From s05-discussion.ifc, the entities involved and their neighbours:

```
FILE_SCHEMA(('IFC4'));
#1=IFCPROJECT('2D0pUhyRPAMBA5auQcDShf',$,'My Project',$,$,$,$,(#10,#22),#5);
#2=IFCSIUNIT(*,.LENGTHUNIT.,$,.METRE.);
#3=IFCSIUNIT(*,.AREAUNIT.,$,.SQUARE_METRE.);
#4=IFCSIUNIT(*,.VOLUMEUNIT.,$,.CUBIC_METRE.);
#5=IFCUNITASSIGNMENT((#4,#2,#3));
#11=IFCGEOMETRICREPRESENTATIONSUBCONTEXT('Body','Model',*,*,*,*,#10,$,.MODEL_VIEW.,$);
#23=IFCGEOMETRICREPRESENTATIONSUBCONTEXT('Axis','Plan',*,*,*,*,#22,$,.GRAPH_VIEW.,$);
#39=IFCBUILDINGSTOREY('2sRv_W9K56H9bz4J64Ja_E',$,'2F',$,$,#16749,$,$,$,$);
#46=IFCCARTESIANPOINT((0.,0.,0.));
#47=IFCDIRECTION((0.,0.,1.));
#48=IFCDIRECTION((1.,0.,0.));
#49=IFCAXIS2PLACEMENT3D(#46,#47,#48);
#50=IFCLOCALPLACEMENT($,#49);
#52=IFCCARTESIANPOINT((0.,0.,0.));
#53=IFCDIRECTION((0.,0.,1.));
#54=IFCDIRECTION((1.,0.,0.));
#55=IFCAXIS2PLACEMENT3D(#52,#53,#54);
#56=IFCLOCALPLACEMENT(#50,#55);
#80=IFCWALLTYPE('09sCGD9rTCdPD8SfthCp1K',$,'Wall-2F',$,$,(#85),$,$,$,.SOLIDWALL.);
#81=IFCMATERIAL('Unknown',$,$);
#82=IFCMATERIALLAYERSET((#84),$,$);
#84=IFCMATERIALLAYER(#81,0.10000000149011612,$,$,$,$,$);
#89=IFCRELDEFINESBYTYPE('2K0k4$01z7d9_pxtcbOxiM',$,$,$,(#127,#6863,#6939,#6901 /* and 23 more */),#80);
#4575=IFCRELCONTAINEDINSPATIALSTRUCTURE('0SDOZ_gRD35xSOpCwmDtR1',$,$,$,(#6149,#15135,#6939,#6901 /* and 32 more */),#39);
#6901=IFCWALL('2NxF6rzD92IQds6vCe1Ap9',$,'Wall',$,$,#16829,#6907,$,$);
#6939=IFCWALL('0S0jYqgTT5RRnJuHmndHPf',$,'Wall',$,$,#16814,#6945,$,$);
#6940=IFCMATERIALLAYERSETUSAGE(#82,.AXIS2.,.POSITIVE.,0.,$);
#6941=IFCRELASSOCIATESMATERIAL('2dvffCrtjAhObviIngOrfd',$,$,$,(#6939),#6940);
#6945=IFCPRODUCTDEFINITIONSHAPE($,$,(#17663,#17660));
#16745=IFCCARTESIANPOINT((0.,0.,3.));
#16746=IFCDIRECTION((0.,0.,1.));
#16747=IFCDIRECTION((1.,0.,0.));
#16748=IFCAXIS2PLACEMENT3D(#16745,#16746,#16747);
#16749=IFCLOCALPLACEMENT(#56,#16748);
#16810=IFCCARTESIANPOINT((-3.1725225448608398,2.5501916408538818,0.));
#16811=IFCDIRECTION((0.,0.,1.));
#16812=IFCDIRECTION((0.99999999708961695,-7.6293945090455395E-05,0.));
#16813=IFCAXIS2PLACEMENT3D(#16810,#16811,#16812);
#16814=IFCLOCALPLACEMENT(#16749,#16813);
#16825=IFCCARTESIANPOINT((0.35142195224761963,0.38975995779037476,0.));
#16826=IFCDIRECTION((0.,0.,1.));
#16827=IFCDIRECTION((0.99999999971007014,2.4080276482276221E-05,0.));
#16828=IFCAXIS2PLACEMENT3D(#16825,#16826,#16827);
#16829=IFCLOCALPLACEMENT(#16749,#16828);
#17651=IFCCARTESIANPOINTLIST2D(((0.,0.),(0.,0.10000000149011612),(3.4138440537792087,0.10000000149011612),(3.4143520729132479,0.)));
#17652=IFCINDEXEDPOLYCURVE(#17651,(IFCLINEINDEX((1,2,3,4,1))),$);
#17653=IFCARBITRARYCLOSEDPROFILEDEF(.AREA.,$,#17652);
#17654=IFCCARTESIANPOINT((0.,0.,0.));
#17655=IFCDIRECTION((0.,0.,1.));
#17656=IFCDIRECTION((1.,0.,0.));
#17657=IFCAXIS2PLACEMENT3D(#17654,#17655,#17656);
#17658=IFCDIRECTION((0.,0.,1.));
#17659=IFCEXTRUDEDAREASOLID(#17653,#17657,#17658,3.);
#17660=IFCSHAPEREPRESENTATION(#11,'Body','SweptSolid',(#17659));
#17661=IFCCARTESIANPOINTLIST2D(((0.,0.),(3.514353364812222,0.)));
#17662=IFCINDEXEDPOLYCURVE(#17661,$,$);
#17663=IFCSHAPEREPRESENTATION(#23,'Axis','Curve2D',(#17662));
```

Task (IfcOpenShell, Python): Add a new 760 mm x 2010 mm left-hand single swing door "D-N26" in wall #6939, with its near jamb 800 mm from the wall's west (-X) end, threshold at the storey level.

```python
import numpy as np
import ifcopenshell
import ifcopenshell.api.feature
import ifcopenshell.api.geometry
import ifcopenshell.api.root
import ifcopenshell.api.spatial
import ifcopenshell.geom
import ifcopenshell.util.element
import ifcopenshell.util.placement
import ifcopenshell.util.representation
import ifcopenshell.util.shape
import ifcopenshell.util.unit

model = ifcopenshell.open("s05-discussion.ifc")
unit_scale = ifcopenshell.util.unit.calculate_unit_scale(model)
settings = ifcopenshell.geom.settings()


def volume(element):
    """Net volume in cubic metres, openings subtracted."""
    shape = ifcopenshell.geom.create_shape(settings, element)
    return ifcopenshell.util.shape.get_volume(shape.geometry)


wall = model.by_id(6939)
storey = ifcopenshell.util.element.get_container(wall, ifc_class="IfcBuildingStorey")
context = ifcopenshell.util.representation.get_context(model, "Model", "Body", "MODEL_VIEW")
before = volume(wall)

width, height, from_end, sill = 0.76, 2.01, 0.8, 0.0  # metres

# The wall runs along its own X axis, and the end named is its -X end.
wall_shape = ifcopenshell.geom.create_shape(settings, wall)
x, y, z = ifcopenshell.util.shape.get_vertices(wall_shape.geometry).T
start = x.min() + from_end
face, thickness = float(y.min()), float(y.max() - y.min())
wall_matrix = ifcopenshell.util.placement.get_local_placement(wall.ObjectPlacement)
level = ifcopenshell.util.placement.get_local_placement(storey.ObjectPlacement)[2, 3]


def in_wall(x, y):
    """Placement at x, y metres in the wall's axes, at sill height."""
    matrix = wall_matrix.copy()
    matrix[:, 3] = wall_matrix @ np.array([x / unit_scale, y / unit_scale, 0.0, 1.0])
    matrix[2, 3] = level + sill / unit_scale
    return matrix


# Opening: a box that overshoots both wall faces by 50 mm.
opening = ifcopenshell.api.root.create_entity(model, ifc_class="IfcOpeningElement", predefined_type="OPENING")
box = ifcopenshell.api.geometry.add_wall_representation(
    model, context=context, length=width, height=height, thickness=thickness + 0.1
)
ifcopenshell.api.geometry.assign_representation(model, product=opening, representation=box)
ifcopenshell.api.geometry.edit_object_placement(model, product=opening, matrix=in_wall(start, face - 0.05), is_si=False)
ifcopenshell.api.feature.add_feature(model, feature=opening, element=wall)

door = ifcopenshell.api.root.create_entity(model, ifc_class="IfcDoor", name="D-N26", predefined_type="DOOR")
door.OverallWidth, door.OverallHeight = width / unit_scale, height / unit_scale
door.OperationType = "SINGLE_SWING_LEFT"
body = ifcopenshell.api.geometry.add_door_representation(
    model,
    context=context,
    overall_width=door.OverallWidth,
    overall_height=door.OverallHeight,
    operation_type="SINGLE_SWING_LEFT",
    lining_properties={"LiningDepth": thickness / unit_scale, "ThresholdDepth": thickness / unit_scale},
)
ifcopenshell.api.geometry.assign_representation(model, product=door, representation=body)
ifcopenshell.api.spatial.assign_container(model, products=[door], relating_structure=storey)
ifcopenshell.api.feature.add_filling(model, opening=opening, element=door)

# The lining spans the wall, so the door starts at the wall face.
ifcopenshell.api.geometry.edit_object_placement(model, product=door, matrix=in_wall(start, face), is_si=False)

after = volume(wall)

print(f"wall volume {before:.3f} -> {after:.3f} m3")

model.write("s05-discussion_rev.ifc")
```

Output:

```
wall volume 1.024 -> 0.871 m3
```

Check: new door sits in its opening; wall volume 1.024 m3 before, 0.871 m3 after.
